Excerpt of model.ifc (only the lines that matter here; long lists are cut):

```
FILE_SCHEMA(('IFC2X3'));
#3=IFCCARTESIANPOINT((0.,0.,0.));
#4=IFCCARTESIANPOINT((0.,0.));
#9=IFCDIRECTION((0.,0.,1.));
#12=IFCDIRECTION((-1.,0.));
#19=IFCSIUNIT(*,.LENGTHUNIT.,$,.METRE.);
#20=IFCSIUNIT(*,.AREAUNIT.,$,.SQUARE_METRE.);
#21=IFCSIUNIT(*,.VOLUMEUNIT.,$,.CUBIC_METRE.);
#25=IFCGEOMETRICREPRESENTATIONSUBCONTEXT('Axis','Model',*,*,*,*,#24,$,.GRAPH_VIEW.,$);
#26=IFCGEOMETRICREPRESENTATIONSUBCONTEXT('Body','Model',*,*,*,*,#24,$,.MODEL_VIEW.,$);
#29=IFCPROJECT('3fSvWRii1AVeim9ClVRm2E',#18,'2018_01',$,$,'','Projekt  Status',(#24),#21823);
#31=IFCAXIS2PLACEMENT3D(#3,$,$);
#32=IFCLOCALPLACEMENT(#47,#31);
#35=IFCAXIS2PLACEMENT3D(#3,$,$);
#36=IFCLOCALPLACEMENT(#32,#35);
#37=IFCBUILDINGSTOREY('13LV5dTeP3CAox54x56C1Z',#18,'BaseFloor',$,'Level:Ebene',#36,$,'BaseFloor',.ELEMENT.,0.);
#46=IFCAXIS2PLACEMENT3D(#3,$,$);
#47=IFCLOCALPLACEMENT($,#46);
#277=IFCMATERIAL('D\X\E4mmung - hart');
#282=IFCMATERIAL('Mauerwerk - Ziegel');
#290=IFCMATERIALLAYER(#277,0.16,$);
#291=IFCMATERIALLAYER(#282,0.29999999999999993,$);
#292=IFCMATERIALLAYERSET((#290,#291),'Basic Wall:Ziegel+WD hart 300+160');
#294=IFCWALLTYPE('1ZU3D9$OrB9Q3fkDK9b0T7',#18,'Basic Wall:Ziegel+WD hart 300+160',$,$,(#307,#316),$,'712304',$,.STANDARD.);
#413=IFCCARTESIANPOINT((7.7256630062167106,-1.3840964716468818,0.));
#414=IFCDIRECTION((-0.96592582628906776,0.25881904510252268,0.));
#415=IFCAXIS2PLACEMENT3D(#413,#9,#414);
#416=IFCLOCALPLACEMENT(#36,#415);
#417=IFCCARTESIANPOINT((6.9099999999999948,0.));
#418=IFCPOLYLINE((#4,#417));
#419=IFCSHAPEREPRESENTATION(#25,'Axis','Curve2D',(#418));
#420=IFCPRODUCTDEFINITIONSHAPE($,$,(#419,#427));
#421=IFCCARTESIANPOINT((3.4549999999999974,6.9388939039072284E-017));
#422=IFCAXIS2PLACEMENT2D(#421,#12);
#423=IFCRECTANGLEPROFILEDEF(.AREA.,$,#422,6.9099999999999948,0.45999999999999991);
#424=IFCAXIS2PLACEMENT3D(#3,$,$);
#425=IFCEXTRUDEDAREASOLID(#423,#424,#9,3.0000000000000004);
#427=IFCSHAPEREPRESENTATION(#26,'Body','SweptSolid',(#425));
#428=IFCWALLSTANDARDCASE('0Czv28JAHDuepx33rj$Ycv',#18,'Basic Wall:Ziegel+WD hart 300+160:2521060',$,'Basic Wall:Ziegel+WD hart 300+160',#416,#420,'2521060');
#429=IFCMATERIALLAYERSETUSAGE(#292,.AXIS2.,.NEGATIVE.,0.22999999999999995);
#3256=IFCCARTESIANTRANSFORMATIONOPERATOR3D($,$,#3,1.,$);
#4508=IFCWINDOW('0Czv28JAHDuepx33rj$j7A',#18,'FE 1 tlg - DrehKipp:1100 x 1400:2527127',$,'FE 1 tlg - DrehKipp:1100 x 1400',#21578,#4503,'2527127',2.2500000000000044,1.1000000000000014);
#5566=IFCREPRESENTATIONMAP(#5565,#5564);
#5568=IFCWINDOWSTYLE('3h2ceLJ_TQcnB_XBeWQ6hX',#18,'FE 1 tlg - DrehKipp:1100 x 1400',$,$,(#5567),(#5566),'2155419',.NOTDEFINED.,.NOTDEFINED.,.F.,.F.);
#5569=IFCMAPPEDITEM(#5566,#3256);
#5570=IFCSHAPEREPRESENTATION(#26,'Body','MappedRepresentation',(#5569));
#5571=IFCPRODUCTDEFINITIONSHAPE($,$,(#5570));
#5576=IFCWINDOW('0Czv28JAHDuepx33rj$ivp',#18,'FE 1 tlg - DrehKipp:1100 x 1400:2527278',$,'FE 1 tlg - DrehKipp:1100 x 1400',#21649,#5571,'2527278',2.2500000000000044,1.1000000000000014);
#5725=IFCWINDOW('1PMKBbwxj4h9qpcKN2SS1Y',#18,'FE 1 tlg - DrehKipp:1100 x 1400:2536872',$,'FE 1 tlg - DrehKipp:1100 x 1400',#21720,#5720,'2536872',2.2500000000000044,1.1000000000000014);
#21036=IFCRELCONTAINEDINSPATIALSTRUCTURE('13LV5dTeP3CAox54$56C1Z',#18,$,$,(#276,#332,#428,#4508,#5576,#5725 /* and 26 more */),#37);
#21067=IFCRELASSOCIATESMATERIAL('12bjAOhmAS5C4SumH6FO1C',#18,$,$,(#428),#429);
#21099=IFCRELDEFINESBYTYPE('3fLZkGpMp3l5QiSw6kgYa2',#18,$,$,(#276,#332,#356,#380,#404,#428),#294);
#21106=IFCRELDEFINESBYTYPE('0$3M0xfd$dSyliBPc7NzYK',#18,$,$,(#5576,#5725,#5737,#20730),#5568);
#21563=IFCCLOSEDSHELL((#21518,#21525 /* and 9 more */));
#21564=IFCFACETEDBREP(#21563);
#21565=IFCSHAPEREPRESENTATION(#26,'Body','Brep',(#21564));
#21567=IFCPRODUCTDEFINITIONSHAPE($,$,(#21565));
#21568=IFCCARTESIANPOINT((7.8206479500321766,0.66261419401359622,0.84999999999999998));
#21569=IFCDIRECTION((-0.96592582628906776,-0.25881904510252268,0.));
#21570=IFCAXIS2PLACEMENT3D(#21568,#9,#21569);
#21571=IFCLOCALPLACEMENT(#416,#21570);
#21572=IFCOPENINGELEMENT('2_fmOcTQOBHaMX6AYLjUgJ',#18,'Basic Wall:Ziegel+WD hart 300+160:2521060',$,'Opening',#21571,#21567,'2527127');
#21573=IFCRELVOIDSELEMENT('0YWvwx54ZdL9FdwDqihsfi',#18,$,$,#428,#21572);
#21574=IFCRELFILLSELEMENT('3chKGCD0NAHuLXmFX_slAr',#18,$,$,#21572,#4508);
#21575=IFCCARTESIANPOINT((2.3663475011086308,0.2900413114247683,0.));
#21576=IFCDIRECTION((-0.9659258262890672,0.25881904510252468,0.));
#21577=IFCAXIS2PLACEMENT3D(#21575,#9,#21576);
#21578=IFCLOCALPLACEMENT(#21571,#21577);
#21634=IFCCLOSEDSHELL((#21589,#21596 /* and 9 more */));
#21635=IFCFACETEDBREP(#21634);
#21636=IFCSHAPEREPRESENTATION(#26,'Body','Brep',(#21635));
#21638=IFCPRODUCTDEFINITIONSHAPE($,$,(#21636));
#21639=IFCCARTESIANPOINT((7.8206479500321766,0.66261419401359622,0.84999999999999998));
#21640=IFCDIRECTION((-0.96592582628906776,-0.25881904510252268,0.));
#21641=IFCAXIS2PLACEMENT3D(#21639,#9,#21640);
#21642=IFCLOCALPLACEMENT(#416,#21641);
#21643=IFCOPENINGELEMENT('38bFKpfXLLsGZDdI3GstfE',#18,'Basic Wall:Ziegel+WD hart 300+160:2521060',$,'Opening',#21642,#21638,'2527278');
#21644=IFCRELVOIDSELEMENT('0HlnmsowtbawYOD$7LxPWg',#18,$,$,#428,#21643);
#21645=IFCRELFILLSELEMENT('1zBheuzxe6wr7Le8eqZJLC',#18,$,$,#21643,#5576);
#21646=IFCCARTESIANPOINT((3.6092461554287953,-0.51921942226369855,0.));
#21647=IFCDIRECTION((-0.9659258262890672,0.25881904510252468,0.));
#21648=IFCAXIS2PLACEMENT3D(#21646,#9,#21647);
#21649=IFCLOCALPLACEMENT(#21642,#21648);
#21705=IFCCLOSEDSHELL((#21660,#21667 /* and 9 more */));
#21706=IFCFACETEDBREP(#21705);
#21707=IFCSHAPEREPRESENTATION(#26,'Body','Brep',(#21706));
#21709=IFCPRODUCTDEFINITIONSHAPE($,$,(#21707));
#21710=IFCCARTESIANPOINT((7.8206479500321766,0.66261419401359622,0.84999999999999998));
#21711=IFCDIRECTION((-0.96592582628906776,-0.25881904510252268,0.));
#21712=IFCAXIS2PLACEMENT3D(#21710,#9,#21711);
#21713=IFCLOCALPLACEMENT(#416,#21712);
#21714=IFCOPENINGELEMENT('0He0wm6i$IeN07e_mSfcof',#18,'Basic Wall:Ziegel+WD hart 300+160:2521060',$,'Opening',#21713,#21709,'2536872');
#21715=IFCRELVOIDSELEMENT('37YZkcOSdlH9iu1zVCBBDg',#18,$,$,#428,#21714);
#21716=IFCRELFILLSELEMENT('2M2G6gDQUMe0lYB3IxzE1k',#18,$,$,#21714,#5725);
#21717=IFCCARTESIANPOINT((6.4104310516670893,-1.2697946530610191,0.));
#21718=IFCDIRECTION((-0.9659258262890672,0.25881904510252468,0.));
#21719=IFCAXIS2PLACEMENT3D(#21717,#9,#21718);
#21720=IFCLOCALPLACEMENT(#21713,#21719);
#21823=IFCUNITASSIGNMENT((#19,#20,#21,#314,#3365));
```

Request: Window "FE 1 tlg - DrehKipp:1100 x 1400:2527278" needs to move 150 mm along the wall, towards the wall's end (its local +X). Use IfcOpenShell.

```python
import ifcopenshell
import ifcopenshell.api.geometry
import ifcopenshell.util.placement
import ifcopenshell.util.unit

model = ifcopenshell.open("model.ifc")
unit_scale = ifcopenshell.util.unit.calculate_unit_scale(model)

window = model.by_guid("0Czv28JAHDuepx33rj$ivp")
opening = window.FillsVoids[0].RelatingOpeningElement
wall = opening.VoidsElements[0].RelatingBuildingElement

wall_matrix = ifcopenshell.util.placement.get_local_placement(wall.ObjectPlacement)
shift = wall_matrix[:3, 0] * 0.15 / unit_scale
before = ifcopenshell.util.placement.get_local_placement(window.ObjectPlacement)[:3, 3].copy()

# The window is placed relative to its opening, so it follows when the opening moves.
matrix = ifcopenshell.util.placement.get_local_placement(opening.ObjectPlacement)
matrix[:3, 3] += shift
ifcopenshell.api.geometry.edit_object_placement(
    model, product=opening, matrix=matrix, is_si=False, should_transform_children=True
)

after = ifcopenshell.util.placement.get_local_placement(window.ObjectPlacement)[:3, 3]
print("window moved by", (after - before).round(3) + 0.0)

model.write("model_updated.ifc")
```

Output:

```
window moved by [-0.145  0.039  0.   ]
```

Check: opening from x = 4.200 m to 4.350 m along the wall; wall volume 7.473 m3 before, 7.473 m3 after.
